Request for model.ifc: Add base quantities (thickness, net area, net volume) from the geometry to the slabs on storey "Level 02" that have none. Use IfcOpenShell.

First a look at what the model holds.

```python
import ifcopenshell
import ifcopenshell.util.element
import ifcopenshell.util.unit

model = ifcopenshell.open("model.ifc")
print(model.schema)
for unit_type in ("LENGTHUNIT", "AREAUNIT", "VOLUMEUNIT"):
    print(unit_type, ifcopenshell.util.unit.calculate_unit_scale(model, unit_type))
storey = next(s for s in model.by_type("IfcBuildingStorey") if s.Name == "Level 02")
slabs = [e for e in ifcopenshell.util.element.get_decomposition(storey) if e.is_a("IfcSlab")]
for e in sorted(slabs, key=lambda e: e.id()):
    print(e.id(), e.is_a(), e.Name, list(ifcopenshell.util.element.get_psets(e, qtos_only=True)), sep=" | ")
```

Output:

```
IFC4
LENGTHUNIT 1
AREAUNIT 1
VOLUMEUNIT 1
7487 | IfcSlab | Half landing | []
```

```python
import ifcopenshell
import ifcopenshell.api.pset
import ifcopenshell.geom
import ifcopenshell.util.element
import ifcopenshell.util.shape
import ifcopenshell.util.unit

model = ifcopenshell.open("model.ifc")
unit_scale = ifcopenshell.util.unit.calculate_unit_scale(model)
area_scale = ifcopenshell.util.unit.calculate_unit_scale(model, "AREAUNIT")
volume_scale = ifcopenshell.util.unit.calculate_unit_scale(model, "VOLUMEUNIT")
settings = ifcopenshell.geom.settings()

storey = next(s for s in model.by_type("IfcBuildingStorey") if s.Name == "Level 02")
slabs = [e for e in ifcopenshell.util.element.get_decomposition(storey) if e.is_a("IfcSlab")]

for e in sorted(slabs, key=lambda e: e.id()):
    if ifcopenshell.util.element.get_psets(e, qtos_only=True, should_inherit=False):
        continue
    # Geometry comes back in metres, in the element's own axes.
    shape = ifcopenshell.geom.create_shape(settings, e)
    values = {
        "Width": ifcopenshell.util.shape.get_z(shape.geometry) / unit_scale,
        "NetArea": ifcopenshell.util.shape.get_footprint_area(shape.geometry) / area_scale,
        "NetVolume": ifcopenshell.util.shape.get_volume(shape.geometry) / volume_scale,
    }
    qto = ifcopenshell.api.pset.add_qto(model, product=e, name="Qto_SlabBaseQuantities")
    ifcopenshell.api.pset.edit_qto(model, qto=qto, properties=values)
    print(e.id(), {k: round(v, 3) for k, v in values.items()})

model.write("model_v2.ifc")
```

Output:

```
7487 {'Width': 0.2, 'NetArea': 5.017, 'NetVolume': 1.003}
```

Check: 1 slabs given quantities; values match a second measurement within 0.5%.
